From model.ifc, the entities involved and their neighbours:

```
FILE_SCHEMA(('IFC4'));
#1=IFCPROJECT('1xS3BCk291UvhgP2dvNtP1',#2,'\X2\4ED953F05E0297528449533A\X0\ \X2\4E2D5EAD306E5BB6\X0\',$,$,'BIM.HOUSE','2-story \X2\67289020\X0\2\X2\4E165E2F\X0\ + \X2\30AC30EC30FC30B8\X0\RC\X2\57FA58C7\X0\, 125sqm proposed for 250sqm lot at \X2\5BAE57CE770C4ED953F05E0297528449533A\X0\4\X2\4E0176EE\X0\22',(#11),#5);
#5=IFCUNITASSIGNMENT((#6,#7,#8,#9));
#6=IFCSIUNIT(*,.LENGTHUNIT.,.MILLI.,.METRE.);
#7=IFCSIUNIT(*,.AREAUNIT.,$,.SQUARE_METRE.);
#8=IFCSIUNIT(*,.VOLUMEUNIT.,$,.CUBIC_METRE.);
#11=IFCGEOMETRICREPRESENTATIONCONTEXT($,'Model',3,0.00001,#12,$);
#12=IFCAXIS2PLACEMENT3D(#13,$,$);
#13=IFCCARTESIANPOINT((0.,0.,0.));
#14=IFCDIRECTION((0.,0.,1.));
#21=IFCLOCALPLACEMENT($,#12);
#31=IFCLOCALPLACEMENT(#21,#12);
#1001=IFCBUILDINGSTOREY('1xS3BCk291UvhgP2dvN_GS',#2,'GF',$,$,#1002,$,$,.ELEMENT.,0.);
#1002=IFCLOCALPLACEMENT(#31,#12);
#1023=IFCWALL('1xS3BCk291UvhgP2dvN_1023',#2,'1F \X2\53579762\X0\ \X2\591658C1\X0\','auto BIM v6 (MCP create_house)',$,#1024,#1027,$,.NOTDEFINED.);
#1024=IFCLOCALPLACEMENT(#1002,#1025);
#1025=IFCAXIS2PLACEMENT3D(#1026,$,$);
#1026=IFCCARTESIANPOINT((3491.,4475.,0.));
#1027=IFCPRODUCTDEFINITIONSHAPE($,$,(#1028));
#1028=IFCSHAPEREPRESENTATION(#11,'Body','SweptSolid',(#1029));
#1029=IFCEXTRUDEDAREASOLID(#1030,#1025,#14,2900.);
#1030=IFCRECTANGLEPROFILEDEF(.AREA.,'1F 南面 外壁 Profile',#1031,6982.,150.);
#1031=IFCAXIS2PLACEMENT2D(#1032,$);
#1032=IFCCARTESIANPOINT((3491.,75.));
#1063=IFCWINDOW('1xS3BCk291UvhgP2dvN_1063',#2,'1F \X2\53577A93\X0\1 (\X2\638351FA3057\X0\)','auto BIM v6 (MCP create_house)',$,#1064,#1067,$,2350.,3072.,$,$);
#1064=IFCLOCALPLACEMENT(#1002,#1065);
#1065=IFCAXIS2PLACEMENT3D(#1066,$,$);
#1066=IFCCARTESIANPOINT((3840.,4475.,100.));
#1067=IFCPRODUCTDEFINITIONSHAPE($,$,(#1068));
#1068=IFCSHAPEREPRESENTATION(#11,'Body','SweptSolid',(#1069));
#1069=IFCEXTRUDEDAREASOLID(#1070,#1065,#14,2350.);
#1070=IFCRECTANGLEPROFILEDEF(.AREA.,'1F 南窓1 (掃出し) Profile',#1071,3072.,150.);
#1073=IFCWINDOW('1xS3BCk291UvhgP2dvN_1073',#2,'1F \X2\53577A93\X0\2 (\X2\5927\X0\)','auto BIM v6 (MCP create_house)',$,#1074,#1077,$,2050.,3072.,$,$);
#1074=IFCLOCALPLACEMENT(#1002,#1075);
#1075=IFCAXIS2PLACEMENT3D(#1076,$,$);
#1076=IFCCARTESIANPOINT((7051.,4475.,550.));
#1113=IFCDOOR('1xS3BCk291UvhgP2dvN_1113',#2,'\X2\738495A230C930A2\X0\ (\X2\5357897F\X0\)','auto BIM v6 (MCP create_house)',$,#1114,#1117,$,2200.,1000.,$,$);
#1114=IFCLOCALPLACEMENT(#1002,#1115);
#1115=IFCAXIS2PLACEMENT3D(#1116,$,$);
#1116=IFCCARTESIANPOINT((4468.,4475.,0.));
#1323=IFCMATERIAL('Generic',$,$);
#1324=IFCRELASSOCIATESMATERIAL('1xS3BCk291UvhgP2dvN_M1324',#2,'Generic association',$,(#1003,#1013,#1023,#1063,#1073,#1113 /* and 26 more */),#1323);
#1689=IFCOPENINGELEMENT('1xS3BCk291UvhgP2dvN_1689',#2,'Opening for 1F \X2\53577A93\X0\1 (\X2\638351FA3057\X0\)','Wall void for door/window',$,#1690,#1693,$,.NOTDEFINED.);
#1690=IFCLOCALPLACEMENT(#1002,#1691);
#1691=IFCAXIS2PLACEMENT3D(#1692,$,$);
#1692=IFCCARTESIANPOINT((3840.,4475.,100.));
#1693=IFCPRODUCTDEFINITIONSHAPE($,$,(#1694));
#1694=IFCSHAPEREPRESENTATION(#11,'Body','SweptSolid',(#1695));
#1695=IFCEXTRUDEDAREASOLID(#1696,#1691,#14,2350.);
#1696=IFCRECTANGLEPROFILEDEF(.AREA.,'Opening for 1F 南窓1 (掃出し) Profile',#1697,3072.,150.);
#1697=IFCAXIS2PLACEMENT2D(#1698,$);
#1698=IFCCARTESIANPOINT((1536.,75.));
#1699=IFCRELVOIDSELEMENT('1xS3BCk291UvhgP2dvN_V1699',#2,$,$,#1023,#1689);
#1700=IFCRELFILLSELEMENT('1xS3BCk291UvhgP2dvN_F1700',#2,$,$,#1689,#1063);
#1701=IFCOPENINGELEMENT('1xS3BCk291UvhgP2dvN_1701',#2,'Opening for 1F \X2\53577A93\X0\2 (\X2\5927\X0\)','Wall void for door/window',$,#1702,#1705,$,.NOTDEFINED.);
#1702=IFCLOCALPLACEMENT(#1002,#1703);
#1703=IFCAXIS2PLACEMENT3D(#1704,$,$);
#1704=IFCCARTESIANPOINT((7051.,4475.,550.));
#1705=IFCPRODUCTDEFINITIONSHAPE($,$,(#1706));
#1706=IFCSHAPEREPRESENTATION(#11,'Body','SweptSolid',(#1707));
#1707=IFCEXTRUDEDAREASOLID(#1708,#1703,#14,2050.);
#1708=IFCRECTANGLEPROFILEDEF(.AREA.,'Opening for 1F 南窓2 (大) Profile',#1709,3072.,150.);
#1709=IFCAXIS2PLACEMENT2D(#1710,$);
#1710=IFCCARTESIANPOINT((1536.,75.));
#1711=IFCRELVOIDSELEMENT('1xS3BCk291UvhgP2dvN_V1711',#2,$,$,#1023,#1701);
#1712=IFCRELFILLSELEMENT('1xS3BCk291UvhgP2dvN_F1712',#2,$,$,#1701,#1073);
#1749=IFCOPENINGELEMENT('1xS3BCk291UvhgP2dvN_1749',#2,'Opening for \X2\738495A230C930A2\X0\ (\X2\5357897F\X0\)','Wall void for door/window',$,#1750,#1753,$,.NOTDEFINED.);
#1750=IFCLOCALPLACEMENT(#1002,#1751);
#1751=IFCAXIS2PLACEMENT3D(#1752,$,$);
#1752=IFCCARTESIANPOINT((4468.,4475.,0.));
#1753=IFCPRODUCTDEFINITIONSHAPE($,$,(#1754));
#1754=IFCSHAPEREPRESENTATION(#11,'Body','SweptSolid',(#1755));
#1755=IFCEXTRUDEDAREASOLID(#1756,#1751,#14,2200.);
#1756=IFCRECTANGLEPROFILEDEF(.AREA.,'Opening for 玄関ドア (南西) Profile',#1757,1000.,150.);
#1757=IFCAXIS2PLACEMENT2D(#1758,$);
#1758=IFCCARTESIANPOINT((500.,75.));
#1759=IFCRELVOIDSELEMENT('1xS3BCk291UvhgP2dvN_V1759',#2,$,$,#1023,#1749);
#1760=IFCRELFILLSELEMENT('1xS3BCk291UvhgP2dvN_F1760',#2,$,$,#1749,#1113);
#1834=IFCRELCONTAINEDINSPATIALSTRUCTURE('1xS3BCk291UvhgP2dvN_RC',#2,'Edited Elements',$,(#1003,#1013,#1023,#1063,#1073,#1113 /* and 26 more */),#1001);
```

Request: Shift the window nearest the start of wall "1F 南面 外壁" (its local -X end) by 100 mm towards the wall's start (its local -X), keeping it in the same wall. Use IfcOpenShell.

```python
import ifcopenshell
import ifcopenshell.api.geometry
import ifcopenshell.util.placement

model = ifcopenshell.open("model.ifc")

window = model.by_id(1063)
opening = window.FillsVoids[0].RelatingOpeningElement
wall = opening.VoidsElements[0].RelatingBuildingElement

wall_matrix = ifcopenshell.util.placement.get_local_placement(wall.ObjectPlacement)
shift = wall_matrix[:3, 0] * -100.0
before = ifcopenshell.util.placement.get_local_placement(window.ObjectPlacement)[:3, 3].copy()

# The window is not placed relative to its opening, so move both.
for product in (opening, window):
    matrix = ifcopenshell.util.placement.get_local_placement(product.ObjectPlacement)
    matrix[:3, 3] += shift
    ifcopenshell.api.geometry.edit_object_placement(model, product=product, matrix=matrix, is_si=False)

after = ifcopenshell.util.placement.get_local_placement(window.ObjectPlacement)[:3, 3]
print("window moved by", (after - before).round(3) + 0.0)

model.write("model_v2.ifc")
```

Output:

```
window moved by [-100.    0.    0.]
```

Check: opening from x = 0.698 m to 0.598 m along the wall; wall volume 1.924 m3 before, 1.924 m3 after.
